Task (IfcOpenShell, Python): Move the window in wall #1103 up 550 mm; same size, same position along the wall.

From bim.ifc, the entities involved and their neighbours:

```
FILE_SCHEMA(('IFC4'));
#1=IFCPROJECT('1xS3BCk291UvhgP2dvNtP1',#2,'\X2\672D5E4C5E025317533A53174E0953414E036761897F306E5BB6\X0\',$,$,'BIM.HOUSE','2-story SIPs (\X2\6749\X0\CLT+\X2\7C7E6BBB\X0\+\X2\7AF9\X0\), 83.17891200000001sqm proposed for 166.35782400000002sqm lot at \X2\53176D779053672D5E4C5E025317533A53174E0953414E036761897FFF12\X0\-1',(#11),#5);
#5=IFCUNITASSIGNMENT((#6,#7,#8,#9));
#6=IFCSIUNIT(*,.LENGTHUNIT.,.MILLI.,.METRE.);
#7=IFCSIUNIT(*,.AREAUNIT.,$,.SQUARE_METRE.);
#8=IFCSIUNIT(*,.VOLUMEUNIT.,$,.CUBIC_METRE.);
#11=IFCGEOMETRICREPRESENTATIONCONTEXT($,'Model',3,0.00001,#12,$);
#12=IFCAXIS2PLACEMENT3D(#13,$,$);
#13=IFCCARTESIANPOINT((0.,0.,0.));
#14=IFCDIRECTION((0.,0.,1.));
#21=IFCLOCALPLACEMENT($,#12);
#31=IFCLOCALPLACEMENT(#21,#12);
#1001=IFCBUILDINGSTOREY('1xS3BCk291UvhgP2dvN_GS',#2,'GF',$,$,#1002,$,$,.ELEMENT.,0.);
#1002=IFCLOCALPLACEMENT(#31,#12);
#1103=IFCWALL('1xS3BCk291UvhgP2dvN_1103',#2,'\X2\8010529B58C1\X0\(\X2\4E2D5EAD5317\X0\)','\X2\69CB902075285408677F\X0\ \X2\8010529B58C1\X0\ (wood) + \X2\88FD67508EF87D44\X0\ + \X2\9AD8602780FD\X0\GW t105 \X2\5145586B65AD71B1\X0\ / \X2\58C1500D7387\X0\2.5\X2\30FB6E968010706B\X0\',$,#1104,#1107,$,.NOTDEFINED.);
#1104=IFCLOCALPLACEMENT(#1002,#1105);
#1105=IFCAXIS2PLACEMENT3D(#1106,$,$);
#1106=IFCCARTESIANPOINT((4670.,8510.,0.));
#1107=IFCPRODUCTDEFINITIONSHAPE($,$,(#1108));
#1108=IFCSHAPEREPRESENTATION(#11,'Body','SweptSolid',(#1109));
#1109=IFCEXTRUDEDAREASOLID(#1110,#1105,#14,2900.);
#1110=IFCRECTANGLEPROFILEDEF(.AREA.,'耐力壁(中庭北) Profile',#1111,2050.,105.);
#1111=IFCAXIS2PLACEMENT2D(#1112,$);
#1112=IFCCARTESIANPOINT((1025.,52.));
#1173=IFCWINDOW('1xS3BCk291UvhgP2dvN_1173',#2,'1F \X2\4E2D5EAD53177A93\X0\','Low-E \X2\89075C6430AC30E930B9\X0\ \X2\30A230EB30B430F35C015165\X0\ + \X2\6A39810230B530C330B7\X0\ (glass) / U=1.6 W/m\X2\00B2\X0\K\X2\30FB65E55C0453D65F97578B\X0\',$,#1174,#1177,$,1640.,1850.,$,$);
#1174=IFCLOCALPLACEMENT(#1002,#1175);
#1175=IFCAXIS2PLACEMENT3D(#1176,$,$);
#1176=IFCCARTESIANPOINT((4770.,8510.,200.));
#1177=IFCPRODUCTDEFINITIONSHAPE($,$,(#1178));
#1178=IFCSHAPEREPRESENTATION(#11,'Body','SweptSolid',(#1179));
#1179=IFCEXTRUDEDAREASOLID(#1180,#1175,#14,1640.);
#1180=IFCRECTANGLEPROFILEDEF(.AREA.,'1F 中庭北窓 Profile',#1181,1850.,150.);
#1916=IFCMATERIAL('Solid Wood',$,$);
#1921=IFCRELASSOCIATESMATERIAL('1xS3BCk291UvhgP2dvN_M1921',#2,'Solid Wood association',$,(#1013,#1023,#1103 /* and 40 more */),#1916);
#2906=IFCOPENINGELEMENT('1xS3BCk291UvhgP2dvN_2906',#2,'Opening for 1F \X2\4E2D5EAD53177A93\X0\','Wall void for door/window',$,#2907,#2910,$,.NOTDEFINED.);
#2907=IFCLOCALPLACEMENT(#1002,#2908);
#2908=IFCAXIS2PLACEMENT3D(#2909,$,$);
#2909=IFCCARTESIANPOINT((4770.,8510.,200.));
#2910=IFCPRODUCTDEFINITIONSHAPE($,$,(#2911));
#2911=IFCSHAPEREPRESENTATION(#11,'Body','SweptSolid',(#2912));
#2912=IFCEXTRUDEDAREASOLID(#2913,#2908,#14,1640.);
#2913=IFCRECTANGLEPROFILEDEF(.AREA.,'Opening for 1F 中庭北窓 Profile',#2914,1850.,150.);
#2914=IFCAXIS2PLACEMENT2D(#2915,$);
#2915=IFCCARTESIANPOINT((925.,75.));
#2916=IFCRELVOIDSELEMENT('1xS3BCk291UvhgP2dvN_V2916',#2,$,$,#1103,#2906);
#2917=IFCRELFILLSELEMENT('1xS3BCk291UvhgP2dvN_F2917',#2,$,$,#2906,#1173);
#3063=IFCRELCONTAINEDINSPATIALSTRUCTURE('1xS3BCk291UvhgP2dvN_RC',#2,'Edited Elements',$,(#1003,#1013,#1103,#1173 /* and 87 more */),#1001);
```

```python
import numpy as np
import ifcopenshell
import ifcopenshell.api.geometry
import ifcopenshell.util.placement
import ifcopenshell.util.unit

model = ifcopenshell.open("bim.ifc")
unit_scale = ifcopenshell.util.unit.calculate_unit_scale(model)

window = model.by_guid("1xS3BCk291UvhgP2dvN_1173")
opening = window.FillsVoids[0].RelatingOpeningElement
dz = 550.0

shift = np.array([0.0, 0.0, dz])
# The window is not placed relative to its opening, so move both.
for product in (opening, window):
    matrix = ifcopenshell.util.placement.get_local_placement(product.ObjectPlacement)
    matrix[:3, 3] += shift
    ifcopenshell.api.geometry.edit_object_placement(model, product=product, matrix=matrix, is_si=False)

print(f"moved by {dz * unit_scale:+.3f} m")

model.write("bim_rev.ifc")
```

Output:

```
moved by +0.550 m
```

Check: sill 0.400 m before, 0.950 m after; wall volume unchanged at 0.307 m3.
